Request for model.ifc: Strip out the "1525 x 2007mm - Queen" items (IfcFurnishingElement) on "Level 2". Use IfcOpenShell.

First a look at what the model holds.

```python
import ifcopenshell
import ifcopenshell.util.element

model = ifcopenshell.open("model.ifc")
print(model.schema)
storey = next(s for s in model.by_type("IfcBuildingStorey") if s.Name == "Level 2")
furniture = [e for e in ifcopenshell.util.element.get_decomposition(storey) if e.is_a("IfcFurnishingElement")]
seen = {}
for e in furniture:
    element_type = ifcopenshell.util.element.get_type(e)
    name = element_type.Name if element_type not in (None, e) else None
    seen[name] = seen.get(name, 0) + 1
for name, count in sorted(seen.items(), key=str):
    print(count, "x", name)
```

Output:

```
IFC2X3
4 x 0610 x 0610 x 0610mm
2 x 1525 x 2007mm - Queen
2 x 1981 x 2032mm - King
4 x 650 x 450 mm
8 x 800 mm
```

```python
import ifcopenshell
import ifcopenshell.api.root
import ifcopenshell.util.element

model = ifcopenshell.open("model.ifc")

storey = next(s for s in model.by_type("IfcBuildingStorey") if s.Name == "Level 2")
furniture = [e for e in ifcopenshell.util.element.get_decomposition(storey) if e.is_a("IfcFurnishingElement")]
targets = [e for e in furniture if (t := ifcopenshell.util.element.get_type(e)) not in (None, e) and t.Name == "1525 x 2007mm - Queen"]

for e in targets:
    ifcopenshell.api.root.remove_product(model, product=e)
print(len(targets), "removed")

model.write("model_rev.ifc")
```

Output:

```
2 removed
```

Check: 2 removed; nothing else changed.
